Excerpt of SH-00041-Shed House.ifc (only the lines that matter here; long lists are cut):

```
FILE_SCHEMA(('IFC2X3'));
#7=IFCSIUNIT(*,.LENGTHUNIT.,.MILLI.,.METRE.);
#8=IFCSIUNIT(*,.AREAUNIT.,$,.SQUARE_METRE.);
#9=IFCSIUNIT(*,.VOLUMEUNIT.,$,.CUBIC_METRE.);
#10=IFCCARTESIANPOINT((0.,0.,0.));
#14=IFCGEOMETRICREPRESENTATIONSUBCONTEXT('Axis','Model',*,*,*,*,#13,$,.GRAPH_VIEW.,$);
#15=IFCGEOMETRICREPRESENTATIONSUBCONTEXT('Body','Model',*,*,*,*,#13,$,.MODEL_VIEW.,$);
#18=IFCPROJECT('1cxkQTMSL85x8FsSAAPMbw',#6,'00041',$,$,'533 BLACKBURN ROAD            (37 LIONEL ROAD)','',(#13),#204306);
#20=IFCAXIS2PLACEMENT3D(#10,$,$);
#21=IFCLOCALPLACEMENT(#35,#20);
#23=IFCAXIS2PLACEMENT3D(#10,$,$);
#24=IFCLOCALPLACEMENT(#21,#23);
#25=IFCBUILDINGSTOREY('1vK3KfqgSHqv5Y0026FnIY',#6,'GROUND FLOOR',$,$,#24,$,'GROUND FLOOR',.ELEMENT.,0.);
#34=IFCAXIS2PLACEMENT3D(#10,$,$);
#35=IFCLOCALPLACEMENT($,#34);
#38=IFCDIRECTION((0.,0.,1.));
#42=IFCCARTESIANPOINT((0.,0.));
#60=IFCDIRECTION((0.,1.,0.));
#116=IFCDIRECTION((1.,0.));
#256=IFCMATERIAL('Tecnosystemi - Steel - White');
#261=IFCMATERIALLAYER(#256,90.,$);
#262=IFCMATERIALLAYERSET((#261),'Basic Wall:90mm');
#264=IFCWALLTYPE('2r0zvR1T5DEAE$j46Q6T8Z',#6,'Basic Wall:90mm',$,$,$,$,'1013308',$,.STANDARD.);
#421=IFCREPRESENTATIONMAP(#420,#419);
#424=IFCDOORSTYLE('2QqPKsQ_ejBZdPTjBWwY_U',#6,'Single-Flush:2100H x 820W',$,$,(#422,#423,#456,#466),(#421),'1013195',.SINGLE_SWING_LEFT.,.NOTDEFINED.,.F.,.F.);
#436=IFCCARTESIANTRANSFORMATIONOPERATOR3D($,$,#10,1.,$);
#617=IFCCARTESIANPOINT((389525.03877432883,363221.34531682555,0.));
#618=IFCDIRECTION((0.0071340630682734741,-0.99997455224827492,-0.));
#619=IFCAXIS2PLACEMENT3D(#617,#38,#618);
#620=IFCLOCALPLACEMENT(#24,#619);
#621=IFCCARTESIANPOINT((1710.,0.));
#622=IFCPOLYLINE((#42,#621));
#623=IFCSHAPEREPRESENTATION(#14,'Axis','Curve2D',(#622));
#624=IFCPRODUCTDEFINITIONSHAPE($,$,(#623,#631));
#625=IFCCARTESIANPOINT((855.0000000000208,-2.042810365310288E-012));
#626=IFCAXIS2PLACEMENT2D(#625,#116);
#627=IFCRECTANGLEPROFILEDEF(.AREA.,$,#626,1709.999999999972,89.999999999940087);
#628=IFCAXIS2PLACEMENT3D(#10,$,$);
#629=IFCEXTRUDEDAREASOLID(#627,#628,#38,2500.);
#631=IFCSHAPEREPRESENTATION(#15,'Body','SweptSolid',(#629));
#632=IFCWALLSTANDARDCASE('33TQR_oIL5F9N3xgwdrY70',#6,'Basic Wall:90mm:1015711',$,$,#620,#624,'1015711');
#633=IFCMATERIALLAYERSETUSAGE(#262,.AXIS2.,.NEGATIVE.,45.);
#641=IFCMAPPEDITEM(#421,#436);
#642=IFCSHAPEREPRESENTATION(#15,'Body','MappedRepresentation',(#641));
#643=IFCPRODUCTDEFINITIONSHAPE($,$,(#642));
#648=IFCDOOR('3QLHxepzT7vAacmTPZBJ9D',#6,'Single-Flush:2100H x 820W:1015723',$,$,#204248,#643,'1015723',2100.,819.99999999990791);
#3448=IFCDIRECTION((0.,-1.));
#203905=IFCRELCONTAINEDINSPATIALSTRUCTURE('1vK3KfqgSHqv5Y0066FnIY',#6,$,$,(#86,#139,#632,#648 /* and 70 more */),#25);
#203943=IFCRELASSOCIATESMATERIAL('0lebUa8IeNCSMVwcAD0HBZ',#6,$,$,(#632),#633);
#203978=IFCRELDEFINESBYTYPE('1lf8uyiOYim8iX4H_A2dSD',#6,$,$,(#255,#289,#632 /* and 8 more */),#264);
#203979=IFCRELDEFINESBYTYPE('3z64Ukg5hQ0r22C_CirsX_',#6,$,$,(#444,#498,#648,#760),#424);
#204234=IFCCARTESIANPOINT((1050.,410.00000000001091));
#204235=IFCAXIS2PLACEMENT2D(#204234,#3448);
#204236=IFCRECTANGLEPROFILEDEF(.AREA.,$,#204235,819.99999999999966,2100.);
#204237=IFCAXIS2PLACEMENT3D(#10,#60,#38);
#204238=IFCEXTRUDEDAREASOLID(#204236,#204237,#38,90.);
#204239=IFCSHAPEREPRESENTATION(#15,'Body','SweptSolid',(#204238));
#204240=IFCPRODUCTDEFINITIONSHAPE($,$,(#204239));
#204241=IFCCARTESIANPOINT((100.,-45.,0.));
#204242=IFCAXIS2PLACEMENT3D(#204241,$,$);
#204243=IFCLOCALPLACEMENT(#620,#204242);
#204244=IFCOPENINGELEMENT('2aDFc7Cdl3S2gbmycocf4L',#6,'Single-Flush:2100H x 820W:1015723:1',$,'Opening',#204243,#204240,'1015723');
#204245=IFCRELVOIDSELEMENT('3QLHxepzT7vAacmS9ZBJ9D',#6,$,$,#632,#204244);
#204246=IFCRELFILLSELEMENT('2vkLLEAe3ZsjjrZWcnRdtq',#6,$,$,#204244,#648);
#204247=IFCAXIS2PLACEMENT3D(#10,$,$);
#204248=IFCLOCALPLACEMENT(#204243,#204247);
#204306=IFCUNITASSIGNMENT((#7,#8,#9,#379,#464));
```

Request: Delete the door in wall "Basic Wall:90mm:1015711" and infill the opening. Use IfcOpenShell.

```python
import ifcopenshell
import ifcopenshell.api.feature
import ifcopenshell.api.root
import ifcopenshell.geom
import ifcopenshell.util.shape

model = ifcopenshell.open("SH-00041-Shed House.ifc")
settings = ifcopenshell.geom.settings()


def volume(element):
    """Net volume in cubic metres, openings subtracted."""
    shape = ifcopenshell.geom.create_shape(settings, element)
    return ifcopenshell.util.shape.get_volume(shape.geometry)


door = model.by_guid("3QLHxepzT7vAacmTPZBJ9D")
opening = door.FillsVoids[0].RelatingOpeningElement
wall = opening.VoidsElements[0].RelatingBuildingElement
before = volume(wall)

ifcopenshell.api.root.remove_product(model, product=door)
ifcopenshell.api.feature.remove_feature(model, feature=opening)

after = volume(wall)

print(f"wall volume {before:.3f} -> {after:.3f} m3")

model.write("SH-00041-Shed House_rev.ifc")
```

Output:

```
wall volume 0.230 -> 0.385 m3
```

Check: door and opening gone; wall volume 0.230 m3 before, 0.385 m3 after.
